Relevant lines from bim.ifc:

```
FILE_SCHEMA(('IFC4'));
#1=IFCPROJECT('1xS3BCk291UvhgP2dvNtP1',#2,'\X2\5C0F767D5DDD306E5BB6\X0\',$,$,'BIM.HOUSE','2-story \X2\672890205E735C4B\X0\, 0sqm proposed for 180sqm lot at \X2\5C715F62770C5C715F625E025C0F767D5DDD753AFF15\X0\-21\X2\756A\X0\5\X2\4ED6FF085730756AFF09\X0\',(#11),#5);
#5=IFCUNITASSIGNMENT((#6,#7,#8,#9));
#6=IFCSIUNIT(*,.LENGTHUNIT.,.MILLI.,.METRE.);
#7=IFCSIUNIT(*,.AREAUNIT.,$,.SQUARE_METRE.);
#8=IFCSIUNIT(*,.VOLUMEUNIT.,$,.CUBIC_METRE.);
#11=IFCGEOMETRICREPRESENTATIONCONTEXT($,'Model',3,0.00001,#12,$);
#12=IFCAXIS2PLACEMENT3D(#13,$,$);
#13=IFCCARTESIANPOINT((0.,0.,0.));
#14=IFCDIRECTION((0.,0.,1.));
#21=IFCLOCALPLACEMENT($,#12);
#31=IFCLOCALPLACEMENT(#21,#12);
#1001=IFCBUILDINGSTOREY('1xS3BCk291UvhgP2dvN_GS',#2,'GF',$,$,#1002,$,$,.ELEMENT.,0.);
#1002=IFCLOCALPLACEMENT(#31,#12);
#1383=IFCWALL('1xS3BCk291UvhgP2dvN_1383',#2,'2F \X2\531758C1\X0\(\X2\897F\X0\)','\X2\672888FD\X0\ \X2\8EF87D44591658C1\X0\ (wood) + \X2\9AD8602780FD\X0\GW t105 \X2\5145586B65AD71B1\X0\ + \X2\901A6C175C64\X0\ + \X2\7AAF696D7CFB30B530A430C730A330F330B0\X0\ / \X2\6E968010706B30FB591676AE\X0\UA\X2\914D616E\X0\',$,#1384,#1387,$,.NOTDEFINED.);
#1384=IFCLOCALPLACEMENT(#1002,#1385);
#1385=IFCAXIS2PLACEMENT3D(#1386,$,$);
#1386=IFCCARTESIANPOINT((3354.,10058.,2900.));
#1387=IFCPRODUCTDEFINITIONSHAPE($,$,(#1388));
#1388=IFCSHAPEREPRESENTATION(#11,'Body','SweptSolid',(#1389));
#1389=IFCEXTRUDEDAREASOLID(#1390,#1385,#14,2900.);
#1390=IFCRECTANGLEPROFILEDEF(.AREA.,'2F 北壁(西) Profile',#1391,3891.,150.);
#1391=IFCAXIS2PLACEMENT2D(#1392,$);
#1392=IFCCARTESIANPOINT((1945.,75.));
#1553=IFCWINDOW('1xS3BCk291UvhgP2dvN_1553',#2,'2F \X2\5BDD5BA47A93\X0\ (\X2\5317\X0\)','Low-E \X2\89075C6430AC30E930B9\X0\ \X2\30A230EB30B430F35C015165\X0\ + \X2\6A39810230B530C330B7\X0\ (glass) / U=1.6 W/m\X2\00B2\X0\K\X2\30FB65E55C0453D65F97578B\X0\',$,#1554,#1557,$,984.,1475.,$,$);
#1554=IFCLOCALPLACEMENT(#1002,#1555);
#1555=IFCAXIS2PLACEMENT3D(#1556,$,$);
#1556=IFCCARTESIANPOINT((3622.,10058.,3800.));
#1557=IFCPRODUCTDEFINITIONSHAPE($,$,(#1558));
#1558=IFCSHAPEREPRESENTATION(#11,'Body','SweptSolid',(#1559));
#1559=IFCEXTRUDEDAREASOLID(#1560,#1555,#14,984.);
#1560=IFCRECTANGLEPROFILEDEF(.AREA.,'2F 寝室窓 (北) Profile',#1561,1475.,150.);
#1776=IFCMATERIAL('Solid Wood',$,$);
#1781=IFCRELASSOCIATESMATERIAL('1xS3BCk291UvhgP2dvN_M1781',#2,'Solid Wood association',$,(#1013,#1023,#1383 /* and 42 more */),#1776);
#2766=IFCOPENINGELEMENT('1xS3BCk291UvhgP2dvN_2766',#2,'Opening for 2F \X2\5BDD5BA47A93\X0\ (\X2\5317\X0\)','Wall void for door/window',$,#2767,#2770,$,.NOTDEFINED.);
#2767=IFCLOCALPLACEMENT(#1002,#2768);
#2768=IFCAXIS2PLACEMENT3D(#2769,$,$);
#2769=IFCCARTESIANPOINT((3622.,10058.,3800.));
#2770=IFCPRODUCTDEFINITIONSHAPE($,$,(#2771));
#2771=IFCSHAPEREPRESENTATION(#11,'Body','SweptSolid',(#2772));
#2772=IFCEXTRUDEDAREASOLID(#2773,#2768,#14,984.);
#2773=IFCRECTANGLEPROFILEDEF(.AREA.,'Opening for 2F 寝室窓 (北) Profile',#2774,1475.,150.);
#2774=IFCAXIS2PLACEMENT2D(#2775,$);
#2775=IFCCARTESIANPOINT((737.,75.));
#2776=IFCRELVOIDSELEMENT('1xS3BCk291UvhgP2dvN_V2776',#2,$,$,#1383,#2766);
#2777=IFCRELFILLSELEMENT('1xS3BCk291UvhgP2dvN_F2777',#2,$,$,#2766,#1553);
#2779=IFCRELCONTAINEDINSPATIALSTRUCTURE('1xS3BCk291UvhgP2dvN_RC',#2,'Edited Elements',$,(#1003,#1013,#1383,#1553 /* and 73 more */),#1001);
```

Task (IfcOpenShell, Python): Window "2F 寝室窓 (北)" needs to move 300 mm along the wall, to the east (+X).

```python
import ifcopenshell
import ifcopenshell.api.geometry
import ifcopenshell.util.placement
import ifcopenshell.util.unit

model = ifcopenshell.open("bim.ifc")
unit_scale = ifcopenshell.util.unit.calculate_unit_scale(model)

window = model.by_guid("1xS3BCk291UvhgP2dvN_1553")
opening = window.FillsVoids[0].RelatingOpeningElement
wall = opening.VoidsElements[0].RelatingBuildingElement

wall_matrix = ifcopenshell.util.placement.get_local_placement(wall.ObjectPlacement)
shift = wall_matrix[:3, 0] * 0.3 / unit_scale
before = ifcopenshell.util.placement.get_local_placement(window.ObjectPlacement)[:3, 3].copy()

# The window is not placed relative to its opening, so move both.
for product in (opening, window):
    matrix = ifcopenshell.util.placement.get_local_placement(product.ObjectPlacement)
    matrix[:3, 3] += shift
    ifcopenshell.api.geometry.edit_object_placement(model, product=product, matrix=matrix, is_si=False)

after = ifcopenshell.util.placement.get_local_placement(window.ObjectPlacement)[:3, 3]
print("window moved by", (after - before).round(3) + 0.0)

model.write("bim_v2.ifc")
```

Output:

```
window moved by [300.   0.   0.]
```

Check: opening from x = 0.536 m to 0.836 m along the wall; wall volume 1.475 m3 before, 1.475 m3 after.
